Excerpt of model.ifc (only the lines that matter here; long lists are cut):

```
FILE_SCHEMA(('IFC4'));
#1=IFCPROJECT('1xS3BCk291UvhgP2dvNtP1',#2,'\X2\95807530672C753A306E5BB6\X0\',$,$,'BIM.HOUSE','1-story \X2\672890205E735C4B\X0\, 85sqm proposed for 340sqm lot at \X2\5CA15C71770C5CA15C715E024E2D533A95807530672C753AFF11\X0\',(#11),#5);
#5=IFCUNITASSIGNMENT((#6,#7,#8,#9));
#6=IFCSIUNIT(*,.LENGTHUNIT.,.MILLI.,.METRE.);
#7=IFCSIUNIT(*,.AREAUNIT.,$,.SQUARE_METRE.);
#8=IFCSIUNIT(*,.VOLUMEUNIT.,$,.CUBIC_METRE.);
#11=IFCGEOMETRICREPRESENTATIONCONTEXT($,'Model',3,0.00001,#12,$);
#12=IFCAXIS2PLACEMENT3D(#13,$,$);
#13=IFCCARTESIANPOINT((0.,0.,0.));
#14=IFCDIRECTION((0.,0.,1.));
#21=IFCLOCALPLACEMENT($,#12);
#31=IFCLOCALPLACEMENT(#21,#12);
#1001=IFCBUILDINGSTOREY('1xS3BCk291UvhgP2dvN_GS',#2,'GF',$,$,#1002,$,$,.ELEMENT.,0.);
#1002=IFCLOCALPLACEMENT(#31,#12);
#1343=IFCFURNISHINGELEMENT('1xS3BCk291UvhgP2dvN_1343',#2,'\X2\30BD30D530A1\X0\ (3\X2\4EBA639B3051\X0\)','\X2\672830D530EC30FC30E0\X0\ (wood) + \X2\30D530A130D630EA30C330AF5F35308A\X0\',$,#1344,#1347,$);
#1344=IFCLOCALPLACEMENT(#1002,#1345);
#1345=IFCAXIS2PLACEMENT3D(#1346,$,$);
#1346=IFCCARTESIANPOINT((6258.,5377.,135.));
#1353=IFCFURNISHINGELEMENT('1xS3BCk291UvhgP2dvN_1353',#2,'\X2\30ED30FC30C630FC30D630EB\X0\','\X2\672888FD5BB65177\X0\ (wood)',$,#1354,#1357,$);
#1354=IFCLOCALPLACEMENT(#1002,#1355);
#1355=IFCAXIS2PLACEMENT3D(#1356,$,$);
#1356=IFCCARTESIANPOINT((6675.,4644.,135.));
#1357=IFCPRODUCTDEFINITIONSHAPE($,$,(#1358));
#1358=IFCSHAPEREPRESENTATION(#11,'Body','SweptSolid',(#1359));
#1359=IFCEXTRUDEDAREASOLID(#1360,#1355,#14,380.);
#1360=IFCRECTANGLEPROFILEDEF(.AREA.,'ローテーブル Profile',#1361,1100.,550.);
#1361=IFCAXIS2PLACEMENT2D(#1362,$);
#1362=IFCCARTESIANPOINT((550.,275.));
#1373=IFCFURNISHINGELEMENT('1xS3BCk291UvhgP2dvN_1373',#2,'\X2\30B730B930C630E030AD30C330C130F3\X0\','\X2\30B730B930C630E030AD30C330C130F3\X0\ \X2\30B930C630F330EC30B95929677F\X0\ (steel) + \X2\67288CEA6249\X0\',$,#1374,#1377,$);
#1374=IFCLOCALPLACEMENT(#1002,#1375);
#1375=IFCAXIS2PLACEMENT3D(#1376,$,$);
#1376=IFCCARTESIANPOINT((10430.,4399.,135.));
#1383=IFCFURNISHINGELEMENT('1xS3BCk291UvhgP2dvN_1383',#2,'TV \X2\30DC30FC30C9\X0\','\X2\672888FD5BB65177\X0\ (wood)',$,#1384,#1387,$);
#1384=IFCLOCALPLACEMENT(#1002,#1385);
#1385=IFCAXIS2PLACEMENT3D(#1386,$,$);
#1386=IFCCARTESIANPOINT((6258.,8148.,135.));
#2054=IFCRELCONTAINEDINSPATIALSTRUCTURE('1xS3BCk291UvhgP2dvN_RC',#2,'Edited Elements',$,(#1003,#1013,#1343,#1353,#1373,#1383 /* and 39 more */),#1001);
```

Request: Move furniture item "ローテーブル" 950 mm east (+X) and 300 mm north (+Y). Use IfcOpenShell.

```python
import ifcopenshell
import ifcopenshell.api.geometry
import ifcopenshell.util.placement
import ifcopenshell.util.unit

model = ifcopenshell.open("model.ifc")
unit_scale = ifcopenshell.util.unit.calculate_unit_scale(model)

item = model.by_guid("1xS3BCk291UvhgP2dvN_1353")
matrix = ifcopenshell.util.placement.get_local_placement(item.ObjectPlacement)
matrix[0, 3] += 0.95 / unit_scale
matrix[1, 3] += 0.3 / unit_scale
ifcopenshell.api.geometry.edit_object_placement(model, product=item, matrix=matrix, is_si=False)

print(ifcopenshell.util.placement.get_local_placement(item.ObjectPlacement).round(3) + 0.0)

model.write("model_edited.ifc")
```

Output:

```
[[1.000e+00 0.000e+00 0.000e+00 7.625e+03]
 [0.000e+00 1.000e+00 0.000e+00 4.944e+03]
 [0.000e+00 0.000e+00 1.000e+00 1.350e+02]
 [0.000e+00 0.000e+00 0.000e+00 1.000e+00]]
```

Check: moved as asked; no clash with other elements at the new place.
